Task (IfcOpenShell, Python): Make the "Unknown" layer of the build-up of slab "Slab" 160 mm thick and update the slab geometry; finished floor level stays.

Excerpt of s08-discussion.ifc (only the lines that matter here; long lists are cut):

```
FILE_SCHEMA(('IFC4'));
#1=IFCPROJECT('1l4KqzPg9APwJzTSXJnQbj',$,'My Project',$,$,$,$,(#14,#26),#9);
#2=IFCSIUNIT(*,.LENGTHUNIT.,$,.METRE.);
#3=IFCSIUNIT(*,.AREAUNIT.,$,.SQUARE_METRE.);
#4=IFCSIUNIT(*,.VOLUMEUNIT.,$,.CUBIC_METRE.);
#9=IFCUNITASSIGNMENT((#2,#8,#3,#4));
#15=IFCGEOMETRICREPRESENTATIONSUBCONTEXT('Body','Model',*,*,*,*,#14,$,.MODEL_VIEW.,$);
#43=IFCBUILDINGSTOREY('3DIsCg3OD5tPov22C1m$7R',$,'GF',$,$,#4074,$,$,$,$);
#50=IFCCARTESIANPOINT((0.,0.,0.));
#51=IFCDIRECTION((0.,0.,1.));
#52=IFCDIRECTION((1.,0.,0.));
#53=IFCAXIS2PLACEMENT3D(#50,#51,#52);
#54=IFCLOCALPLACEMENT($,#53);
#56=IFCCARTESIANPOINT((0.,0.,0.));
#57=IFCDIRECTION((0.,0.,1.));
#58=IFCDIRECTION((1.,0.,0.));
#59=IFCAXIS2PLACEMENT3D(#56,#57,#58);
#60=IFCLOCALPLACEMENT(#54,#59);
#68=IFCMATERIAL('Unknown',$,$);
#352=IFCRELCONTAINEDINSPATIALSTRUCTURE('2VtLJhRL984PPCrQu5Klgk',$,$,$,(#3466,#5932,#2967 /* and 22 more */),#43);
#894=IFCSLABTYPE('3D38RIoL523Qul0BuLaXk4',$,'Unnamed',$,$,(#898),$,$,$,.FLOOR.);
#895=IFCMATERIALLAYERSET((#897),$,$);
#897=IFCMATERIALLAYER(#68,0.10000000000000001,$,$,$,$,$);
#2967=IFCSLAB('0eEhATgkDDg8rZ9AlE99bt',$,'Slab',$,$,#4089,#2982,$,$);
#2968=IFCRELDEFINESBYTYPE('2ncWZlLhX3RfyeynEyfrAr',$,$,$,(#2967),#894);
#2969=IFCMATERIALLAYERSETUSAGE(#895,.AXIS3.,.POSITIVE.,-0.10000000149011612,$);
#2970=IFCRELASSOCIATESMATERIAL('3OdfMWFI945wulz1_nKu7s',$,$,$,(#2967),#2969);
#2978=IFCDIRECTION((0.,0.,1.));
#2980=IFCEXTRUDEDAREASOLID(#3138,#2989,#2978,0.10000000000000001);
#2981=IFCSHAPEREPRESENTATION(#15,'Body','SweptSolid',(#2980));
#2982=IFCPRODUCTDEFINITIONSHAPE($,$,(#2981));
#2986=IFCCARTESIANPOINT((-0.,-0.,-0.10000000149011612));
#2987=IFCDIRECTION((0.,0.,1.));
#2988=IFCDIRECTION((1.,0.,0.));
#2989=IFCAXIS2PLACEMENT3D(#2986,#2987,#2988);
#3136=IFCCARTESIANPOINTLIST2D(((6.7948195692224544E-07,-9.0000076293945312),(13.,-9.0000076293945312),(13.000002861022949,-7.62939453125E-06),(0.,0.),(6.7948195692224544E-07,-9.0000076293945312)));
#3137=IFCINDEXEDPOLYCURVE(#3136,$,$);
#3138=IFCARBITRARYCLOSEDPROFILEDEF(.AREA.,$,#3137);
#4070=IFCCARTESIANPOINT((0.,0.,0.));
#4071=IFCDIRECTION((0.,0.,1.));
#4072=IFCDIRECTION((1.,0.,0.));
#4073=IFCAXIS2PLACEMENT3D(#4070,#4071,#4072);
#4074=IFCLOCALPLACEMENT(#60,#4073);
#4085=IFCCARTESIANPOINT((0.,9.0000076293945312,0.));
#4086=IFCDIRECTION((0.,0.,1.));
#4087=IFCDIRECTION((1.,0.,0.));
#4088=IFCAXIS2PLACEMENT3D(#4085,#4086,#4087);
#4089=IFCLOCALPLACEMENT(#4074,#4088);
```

```python
import ifcopenshell
import ifcopenshell.util.element
import ifcopenshell.util.representation
import ifcopenshell.util.unit

model = ifcopenshell.open("s08-discussion.ifc")
unit_scale = ifcopenshell.util.unit.calculate_unit_scale(model)

layer_set = model.by_id(895)
layer = next(l for l in layer_set.MaterialLayers if l.Material and l.Material.Name == "Unknown")
change = 0.16 / unit_scale - layer.LayerThickness
layer.LayerThickness += change

# Geometry does not follow the layer set by itself.
slabs = [e for e in ifcopenshell.util.element.get_elements_by_material(model, layer_set) if e.is_a("IfcSlab")]
for slab in sorted(slabs, key=lambda e: e.id()):
    body = ifcopenshell.util.representation.get_representation(slab, "Model", "Body")
    solid = body.Items[0]
    old_depth = solid.Depth
    solid.Depth += change
    # Extruded upwards: lower the start of the extrusion so the top stays.
    x, y, z = solid.Position.Location.Coordinates
    solid.Position.Location = model.createIfcCartesianPoint((x, y, z - change))
    print(slab.id(), f"{old_depth:g} -> {solid.Depth:g}")

# The layers are counted up from the underside, which has moved.
for usage in {ifcopenshell.util.element.get_material(slab) for slab in slabs}:
    usage.OffsetFromReferenceLine -= change

model.write("s08-discussion-out.ifc")
```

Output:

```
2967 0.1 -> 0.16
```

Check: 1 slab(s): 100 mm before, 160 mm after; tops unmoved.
